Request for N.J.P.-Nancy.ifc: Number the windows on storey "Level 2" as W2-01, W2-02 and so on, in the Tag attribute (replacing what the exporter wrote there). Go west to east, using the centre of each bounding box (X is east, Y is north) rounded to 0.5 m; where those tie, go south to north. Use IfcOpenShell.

First a look at what the model holds.

```python
import ifcopenshell
import ifcopenshell.util.element
import ifcopenshell.util.placement

model = ifcopenshell.open("N.J.P.-Nancy.ifc")
print(model.schema)
storey = next(s for s in model.by_type("IfcBuildingStorey") if s.Name == "Level 2")
windows = [e for e in ifcopenshell.util.element.get_decomposition(storey) if e.is_a("IfcWindow")]
for e in sorted(windows, key=lambda e: e.id()):
    origin = ifcopenshell.util.placement.get_local_placement(e.ObjectPlacement)[:3, 3]
    print(e.id(), e.Tag, e.Name, origin.round(2) + 0.0, sep=" | ")
```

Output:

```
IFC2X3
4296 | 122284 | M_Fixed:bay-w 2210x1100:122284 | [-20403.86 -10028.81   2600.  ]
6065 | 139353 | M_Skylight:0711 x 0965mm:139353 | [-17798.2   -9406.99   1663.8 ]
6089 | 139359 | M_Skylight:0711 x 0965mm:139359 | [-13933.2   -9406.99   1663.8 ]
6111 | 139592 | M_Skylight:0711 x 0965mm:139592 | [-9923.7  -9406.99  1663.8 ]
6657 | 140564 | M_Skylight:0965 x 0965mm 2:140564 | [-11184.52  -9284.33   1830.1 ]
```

```python
import ifcopenshell
import ifcopenshell.geom
import ifcopenshell.util.element
import ifcopenshell.util.shape

model = ifcopenshell.open("N.J.P.-Nancy.ifc")
settings = ifcopenshell.geom.settings()
settings.set("use-world-coords", True)


def centre(element):
    shape = ifcopenshell.geom.create_shape(settings, element)
    return ifcopenshell.util.shape.get_bbox_centroid(shape.geometry)


storey = next(s for s in model.by_type("IfcBuildingStorey") if s.Name == "Level 2")
windows = [e for e in ifcopenshell.util.element.get_decomposition(storey) if e.is_a("IfcWindow")]

# Insertion points can sit at a corner or the storey origin, so sort by the geometry (in metres).
centres = {e: centre(e) for e in windows}
windows.sort(key=lambda e: (round(centres[e][0] / 0.5), centres[e][1]))

for i, e in enumerate(windows, start=1):
    number = f"W2-{i:02d}"
    e.Tag = number
    print(e.id(), number)

model.write("N.J.P.-Nancy_edited.ifc")
```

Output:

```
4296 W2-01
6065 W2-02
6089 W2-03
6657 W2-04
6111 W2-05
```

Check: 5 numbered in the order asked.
